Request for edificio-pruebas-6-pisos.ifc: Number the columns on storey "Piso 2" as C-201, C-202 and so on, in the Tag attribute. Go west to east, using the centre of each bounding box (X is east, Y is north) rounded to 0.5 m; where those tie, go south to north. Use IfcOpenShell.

First a look at what the model holds.

```python
import ifcopenshell
import ifcopenshell.util.element
import ifcopenshell.util.placement

model = ifcopenshell.open("edificio-pruebas-6-pisos.ifc")
print(model.schema)
storey = next(s for s in model.by_type("IfcBuildingStorey") if s.Name == "Piso 2")
columns = [e for e in ifcopenshell.util.element.get_decomposition(storey) if e.is_a("IfcColumn")]
for e in sorted(columns, key=lambda e: e.id()):
    origin = ifcopenshell.util.placement.get_local_placement(e.ObjectPlacement)[:3, 3]
    print(e.id(), e.Tag, e.Name, origin.round(2) + 0.0, sep=" | ")
```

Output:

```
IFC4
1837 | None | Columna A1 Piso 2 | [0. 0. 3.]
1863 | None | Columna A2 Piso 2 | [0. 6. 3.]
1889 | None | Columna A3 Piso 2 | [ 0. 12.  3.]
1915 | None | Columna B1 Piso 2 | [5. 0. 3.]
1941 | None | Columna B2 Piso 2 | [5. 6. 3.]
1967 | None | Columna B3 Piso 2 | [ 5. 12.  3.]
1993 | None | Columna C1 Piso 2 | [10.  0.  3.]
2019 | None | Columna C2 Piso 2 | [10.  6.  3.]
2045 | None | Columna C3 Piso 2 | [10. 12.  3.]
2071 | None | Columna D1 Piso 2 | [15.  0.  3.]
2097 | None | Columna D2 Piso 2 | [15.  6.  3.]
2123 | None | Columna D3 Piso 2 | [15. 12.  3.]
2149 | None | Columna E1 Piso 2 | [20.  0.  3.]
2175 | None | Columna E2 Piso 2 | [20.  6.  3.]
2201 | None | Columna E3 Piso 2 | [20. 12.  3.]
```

```python
import ifcopenshell
import ifcopenshell.geom
import ifcopenshell.util.element
import ifcopenshell.util.shape

model = ifcopenshell.open("edificio-pruebas-6-pisos.ifc")
settings = ifcopenshell.geom.settings()
settings.set("use-world-coords", True)


def centre(element):
    shape = ifcopenshell.geom.create_shape(settings, element)
    return ifcopenshell.util.shape.get_bbox_centroid(shape.geometry)


storey = next(s for s in model.by_type("IfcBuildingStorey") if s.Name == "Piso 2")
columns = [e for e in ifcopenshell.util.element.get_decomposition(storey) if e.is_a("IfcColumn")]

# Insertion points can sit at a corner or the storey origin, so sort by the geometry (in metres).
centres = {e: centre(e) for e in columns}
columns.sort(key=lambda e: (round(centres[e][0] / 0.5), centres[e][1]))

for i, e in enumerate(columns, start=1):
    number = f"C-2{i:02d}"
    e.Tag = number
    print(e.id(), number)

model.write("edificio-pruebas-6-pisos_v2.ifc")
```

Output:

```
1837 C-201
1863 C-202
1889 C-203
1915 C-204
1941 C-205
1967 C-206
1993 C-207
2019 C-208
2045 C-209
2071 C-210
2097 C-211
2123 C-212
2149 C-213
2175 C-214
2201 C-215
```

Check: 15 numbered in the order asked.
